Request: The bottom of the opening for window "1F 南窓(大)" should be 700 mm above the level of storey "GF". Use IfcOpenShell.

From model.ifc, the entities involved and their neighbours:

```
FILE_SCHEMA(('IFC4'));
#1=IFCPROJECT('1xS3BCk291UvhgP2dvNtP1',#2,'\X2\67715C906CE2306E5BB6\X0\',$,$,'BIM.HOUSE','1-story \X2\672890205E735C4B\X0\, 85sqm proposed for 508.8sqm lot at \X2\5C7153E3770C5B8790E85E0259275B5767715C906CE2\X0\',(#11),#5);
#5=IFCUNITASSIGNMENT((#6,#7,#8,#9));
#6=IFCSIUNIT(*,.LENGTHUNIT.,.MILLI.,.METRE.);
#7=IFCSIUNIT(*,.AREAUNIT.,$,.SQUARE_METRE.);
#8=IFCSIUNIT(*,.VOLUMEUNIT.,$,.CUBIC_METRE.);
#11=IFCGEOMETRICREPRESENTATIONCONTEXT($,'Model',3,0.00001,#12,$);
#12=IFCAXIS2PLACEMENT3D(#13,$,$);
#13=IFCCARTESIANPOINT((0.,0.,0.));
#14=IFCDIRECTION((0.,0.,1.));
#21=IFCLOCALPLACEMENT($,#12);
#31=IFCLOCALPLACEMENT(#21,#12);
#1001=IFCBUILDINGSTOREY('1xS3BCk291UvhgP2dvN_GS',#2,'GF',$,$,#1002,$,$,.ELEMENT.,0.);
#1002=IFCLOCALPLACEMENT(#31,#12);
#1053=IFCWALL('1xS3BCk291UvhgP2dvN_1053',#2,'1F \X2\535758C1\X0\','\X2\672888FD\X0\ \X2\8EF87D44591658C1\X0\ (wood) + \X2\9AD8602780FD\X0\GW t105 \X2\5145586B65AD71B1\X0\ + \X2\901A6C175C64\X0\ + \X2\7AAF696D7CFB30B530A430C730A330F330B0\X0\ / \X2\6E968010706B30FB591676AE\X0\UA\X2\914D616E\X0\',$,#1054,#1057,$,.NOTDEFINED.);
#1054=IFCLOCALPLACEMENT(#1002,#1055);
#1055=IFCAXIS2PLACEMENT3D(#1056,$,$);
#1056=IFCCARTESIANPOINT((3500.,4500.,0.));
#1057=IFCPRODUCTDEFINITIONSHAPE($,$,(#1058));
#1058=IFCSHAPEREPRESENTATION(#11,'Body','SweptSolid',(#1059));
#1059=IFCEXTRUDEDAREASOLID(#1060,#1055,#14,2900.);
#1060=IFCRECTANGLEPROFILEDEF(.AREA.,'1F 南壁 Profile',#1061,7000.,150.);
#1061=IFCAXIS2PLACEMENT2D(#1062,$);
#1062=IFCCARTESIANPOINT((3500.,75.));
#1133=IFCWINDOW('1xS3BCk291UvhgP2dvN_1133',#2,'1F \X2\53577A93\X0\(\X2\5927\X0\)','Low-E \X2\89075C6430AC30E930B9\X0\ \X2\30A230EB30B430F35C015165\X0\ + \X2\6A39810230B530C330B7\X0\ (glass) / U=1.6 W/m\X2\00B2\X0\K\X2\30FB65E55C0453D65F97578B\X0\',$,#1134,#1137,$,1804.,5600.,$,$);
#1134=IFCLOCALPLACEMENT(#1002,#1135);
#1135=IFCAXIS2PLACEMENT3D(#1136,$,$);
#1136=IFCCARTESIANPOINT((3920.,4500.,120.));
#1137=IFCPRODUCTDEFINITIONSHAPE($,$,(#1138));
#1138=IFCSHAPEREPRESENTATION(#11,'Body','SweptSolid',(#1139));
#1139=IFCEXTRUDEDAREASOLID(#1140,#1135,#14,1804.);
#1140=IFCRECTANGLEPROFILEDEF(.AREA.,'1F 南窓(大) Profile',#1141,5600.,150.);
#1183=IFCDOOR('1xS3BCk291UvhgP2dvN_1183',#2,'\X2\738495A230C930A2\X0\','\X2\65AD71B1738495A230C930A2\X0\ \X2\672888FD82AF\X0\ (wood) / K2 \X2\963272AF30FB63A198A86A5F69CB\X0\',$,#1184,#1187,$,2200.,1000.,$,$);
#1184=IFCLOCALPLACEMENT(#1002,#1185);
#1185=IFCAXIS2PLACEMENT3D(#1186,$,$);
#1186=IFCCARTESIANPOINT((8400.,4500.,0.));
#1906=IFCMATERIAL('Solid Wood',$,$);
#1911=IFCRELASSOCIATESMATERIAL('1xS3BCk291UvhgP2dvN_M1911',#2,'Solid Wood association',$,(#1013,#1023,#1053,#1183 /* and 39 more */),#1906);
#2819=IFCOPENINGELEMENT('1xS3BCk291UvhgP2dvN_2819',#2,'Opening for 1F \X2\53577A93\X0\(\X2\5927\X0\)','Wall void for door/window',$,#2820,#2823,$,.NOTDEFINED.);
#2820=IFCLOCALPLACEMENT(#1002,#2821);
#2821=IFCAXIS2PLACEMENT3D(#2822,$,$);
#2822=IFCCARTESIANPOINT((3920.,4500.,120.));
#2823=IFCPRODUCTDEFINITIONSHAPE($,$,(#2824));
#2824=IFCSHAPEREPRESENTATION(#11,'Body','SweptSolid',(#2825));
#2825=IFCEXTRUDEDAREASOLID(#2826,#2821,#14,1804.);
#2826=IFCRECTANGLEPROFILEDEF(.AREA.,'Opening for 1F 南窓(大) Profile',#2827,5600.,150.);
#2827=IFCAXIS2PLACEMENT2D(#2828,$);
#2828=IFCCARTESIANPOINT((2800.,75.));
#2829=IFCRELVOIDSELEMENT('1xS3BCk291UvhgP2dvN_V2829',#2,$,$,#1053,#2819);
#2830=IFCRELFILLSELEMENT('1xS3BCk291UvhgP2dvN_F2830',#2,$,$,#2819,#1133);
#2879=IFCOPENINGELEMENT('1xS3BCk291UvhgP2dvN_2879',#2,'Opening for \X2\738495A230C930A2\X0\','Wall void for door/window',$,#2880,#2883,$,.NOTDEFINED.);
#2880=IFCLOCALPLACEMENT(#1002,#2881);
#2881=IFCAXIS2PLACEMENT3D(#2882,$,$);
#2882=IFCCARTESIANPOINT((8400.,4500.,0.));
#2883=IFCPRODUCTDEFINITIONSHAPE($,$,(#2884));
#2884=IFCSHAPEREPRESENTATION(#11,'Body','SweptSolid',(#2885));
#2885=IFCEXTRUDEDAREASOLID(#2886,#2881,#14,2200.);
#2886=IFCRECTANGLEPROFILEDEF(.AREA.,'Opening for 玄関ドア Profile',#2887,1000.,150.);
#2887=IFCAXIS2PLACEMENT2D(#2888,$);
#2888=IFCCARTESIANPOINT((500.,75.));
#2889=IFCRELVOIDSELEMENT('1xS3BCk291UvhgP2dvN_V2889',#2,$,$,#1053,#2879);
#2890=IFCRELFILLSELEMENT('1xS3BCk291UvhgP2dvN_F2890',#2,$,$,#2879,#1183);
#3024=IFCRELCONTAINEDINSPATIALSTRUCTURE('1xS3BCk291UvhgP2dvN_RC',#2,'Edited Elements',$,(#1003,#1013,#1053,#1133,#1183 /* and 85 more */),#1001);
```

```python
import numpy as np
import ifcopenshell
import ifcopenshell.api.geometry
import ifcopenshell.geom
import ifcopenshell.util.element
import ifcopenshell.util.placement
import ifcopenshell.util.shape
import ifcopenshell.util.unit

model = ifcopenshell.open("model.ifc")
unit_scale = ifcopenshell.util.unit.calculate_unit_scale(model)

window = model.by_guid("1xS3BCk291UvhgP2dvN_1133")
opening = window.FillsVoids[0].RelatingOpeningElement
storey = ifcopenshell.util.element.get_container(window, ifc_class="IfcBuildingStorey")
level = ifcopenshell.util.placement.get_local_placement(storey.ObjectPlacement)[2, 3]

# The opening's origin need not be at the sill, so measure its lowest point.
shape = ifcopenshell.geom.create_shape(ifcopenshell.geom.settings(), opening)
bottom = ifcopenshell.util.shape.get_shape_bottom_elevation(shape, shape.geometry) / unit_scale
dz = level + 700.0 - bottom

shift = np.array([0.0, 0.0, dz])
# The window is not placed relative to its opening, so move both.
for product in (opening, window):
    matrix = ifcopenshell.util.placement.get_local_placement(product.ObjectPlacement)
    matrix[:3, 3] += shift
    ifcopenshell.api.geometry.edit_object_placement(model, product=product, matrix=matrix, is_si=False)

print(f"moved by {dz * unit_scale:+.3f} m")

model.write("model_updated.ifc")
```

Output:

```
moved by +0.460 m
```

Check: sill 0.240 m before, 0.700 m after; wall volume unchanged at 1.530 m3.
